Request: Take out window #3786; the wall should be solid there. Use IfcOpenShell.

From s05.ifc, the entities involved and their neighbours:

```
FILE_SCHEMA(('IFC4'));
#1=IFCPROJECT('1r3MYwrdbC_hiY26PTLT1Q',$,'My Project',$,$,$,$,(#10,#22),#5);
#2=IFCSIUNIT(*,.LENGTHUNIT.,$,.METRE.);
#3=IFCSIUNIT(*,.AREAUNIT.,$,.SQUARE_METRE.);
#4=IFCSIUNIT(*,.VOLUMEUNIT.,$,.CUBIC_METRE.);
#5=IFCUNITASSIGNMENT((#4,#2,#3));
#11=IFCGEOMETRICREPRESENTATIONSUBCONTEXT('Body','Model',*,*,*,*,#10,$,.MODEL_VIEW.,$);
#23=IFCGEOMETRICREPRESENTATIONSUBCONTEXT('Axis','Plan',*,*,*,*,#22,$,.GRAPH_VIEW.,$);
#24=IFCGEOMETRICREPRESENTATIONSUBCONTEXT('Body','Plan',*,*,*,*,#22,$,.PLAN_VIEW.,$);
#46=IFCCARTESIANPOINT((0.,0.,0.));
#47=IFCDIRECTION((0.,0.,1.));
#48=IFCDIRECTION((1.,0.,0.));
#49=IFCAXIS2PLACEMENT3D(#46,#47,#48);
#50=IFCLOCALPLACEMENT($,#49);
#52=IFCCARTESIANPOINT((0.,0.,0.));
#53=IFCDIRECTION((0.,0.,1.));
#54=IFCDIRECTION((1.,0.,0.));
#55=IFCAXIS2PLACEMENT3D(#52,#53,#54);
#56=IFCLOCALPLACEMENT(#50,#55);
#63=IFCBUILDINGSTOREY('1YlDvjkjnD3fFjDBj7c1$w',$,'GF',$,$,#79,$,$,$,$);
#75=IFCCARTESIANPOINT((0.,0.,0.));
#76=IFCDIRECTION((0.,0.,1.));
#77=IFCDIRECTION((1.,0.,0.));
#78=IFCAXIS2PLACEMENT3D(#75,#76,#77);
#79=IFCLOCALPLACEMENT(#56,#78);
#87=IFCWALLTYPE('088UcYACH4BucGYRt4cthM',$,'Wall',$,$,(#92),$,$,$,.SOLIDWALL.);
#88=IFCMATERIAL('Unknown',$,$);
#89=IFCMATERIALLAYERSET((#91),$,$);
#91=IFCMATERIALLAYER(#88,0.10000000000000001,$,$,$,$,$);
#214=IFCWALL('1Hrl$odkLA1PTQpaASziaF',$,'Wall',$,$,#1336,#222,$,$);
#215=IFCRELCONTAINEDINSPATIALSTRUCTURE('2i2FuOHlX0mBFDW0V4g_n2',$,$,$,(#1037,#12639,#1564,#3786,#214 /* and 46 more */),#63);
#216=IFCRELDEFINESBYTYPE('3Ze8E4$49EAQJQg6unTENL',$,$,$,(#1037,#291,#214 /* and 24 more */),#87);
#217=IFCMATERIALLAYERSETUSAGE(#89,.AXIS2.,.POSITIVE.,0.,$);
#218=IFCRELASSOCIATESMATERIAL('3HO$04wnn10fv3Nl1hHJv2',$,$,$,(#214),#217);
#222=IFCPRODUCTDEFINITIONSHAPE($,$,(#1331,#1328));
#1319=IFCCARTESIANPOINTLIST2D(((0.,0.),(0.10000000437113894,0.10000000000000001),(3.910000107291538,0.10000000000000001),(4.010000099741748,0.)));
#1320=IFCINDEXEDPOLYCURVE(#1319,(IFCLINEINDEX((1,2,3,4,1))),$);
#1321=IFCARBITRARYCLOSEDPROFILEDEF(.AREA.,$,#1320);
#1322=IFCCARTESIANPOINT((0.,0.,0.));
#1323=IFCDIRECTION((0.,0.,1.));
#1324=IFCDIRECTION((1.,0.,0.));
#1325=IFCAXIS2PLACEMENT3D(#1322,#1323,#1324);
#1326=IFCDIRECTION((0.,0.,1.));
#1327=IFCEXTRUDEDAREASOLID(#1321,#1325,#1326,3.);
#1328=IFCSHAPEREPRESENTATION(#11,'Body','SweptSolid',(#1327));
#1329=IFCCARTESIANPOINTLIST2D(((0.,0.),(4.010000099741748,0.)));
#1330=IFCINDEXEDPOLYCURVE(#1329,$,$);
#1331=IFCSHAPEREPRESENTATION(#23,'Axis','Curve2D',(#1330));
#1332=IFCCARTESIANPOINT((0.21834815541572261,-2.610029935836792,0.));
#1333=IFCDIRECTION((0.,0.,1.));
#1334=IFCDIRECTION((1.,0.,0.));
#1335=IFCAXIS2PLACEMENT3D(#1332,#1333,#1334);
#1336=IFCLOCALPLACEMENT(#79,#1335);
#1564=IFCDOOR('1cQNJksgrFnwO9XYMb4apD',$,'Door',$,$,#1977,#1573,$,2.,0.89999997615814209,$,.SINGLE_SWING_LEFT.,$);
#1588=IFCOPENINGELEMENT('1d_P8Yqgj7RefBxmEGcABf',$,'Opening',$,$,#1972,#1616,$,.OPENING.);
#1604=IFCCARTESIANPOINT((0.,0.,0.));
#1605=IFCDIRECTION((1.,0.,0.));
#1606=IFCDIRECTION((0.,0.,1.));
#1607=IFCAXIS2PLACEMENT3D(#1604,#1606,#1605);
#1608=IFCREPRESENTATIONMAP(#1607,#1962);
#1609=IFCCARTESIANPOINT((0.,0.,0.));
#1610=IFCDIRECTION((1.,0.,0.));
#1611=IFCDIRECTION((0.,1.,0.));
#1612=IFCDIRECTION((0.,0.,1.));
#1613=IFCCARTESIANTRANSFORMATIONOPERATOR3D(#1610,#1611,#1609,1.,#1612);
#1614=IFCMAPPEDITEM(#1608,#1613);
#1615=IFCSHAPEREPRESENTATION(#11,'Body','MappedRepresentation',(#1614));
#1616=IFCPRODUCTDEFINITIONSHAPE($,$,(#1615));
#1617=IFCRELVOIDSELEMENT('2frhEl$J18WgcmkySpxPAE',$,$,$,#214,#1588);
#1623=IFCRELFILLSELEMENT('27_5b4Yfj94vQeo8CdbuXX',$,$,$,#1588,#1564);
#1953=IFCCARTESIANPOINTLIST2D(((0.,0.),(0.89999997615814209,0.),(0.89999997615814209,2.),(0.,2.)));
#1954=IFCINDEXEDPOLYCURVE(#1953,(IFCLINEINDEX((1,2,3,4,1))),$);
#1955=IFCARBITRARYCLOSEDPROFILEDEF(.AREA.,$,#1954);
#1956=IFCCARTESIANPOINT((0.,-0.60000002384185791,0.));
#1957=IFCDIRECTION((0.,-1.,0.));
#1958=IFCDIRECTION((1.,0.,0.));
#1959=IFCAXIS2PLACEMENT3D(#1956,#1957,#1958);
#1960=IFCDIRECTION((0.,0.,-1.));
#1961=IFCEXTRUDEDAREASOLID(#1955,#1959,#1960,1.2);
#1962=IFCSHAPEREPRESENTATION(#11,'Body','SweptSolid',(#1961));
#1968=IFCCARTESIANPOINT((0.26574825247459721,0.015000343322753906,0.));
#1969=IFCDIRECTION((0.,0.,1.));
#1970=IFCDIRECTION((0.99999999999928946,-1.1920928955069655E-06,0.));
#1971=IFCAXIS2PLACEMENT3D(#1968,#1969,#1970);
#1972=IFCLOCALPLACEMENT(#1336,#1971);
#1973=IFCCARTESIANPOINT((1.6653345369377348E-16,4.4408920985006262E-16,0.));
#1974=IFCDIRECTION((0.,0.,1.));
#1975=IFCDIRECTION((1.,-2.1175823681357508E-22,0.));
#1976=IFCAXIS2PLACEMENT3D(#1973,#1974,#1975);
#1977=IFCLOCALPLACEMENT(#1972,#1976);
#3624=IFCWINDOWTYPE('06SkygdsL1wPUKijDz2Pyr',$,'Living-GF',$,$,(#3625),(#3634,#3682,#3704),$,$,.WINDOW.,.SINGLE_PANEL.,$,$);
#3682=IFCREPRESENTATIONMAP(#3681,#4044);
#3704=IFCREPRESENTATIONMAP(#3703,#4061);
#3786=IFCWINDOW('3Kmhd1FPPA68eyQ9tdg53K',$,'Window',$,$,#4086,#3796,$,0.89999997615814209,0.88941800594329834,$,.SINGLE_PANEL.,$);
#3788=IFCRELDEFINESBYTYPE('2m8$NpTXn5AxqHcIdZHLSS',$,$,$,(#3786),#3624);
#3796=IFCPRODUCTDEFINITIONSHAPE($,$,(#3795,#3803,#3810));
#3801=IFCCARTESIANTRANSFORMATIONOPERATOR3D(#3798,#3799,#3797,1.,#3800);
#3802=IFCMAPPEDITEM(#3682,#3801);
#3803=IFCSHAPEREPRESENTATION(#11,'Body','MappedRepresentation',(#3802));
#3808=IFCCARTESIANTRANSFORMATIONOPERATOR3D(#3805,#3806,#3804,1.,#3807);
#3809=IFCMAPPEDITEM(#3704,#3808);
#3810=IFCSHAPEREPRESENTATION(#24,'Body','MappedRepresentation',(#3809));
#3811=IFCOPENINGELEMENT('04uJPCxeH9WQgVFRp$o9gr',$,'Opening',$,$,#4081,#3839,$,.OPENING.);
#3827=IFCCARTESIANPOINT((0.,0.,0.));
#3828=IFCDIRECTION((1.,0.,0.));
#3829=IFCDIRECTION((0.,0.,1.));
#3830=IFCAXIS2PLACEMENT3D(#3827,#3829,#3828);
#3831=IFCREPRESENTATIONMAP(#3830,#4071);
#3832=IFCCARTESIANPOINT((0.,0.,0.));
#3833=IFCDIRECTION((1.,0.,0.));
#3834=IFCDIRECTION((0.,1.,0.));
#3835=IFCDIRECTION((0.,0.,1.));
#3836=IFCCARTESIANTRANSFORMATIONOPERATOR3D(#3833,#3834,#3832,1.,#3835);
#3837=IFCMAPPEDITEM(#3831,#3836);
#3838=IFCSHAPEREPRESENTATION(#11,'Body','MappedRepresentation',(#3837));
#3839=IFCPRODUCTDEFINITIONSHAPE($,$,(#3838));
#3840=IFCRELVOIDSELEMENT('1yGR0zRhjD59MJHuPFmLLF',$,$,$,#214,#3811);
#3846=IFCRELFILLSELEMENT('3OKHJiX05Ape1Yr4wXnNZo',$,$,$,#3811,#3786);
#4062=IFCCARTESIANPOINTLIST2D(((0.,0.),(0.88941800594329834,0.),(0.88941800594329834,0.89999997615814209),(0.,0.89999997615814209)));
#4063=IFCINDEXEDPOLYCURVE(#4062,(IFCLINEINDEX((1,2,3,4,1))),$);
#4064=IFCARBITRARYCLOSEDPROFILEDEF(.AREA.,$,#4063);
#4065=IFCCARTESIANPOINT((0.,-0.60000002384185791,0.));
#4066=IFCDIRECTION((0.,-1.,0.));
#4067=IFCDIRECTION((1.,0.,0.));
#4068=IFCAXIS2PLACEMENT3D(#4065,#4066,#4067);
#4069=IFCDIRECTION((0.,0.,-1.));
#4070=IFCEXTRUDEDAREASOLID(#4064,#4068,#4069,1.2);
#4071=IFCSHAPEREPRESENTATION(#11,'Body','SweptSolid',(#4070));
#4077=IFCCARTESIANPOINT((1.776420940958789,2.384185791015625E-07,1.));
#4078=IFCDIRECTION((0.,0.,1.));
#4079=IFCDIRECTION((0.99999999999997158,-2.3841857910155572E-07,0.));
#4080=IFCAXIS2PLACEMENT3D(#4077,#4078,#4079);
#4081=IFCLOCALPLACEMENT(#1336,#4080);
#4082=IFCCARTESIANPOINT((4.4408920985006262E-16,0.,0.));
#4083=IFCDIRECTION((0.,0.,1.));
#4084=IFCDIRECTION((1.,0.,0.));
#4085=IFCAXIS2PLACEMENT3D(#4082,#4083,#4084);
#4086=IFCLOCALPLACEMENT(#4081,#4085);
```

```python
import ifcopenshell
import ifcopenshell.api.feature
import ifcopenshell.api.root
import ifcopenshell.geom
import ifcopenshell.util.shape

model = ifcopenshell.open("s05.ifc")
settings = ifcopenshell.geom.settings()


def volume(element):
    """Net volume in cubic metres, openings subtracted."""
    shape = ifcopenshell.geom.create_shape(settings, element)
    return ifcopenshell.util.shape.get_volume(shape.geometry)


window = model.by_guid("3Kmhd1FPPA68eyQ9tdg53K")
opening = window.FillsVoids[0].RelatingOpeningElement
wall = opening.VoidsElements[0].RelatingBuildingElement
before = volume(wall)

ifcopenshell.api.root.remove_product(model, product=window)
ifcopenshell.api.feature.remove_feature(model, feature=opening)

after = volume(wall)

print(f"wall volume {before:.3f} -> {after:.3f} m3")

model.write("s05_edited.ifc")
```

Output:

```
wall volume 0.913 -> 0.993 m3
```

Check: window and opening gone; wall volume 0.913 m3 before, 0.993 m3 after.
